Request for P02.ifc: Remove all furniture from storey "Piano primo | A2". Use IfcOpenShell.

First a look at what the model holds.

```python
import ifcopenshell
import ifcopenshell.util.element

model = ifcopenshell.open("P02.ifc")
print(model.schema)
storey = next(s for s in model.by_type("IfcBuildingStorey") if s.Name == "Piano primo | A2")
furniture = [e for e in ifcopenshell.util.element.get_decomposition(storey) if e.is_a("IfcFurnishingElement")]
seen = {}
for e in furniture:
    element_type = ifcopenshell.util.element.get_type(e)
    name = element_type.Name if element_type not in (None, e) else None
    seen[name] = seen.get(name, 0) + 1
for name, count in sorted(seen.items(), key=str):
    print(count, "x", name)
```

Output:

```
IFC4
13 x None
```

```python
import ifcopenshell
import ifcopenshell.api.root
import ifcopenshell.util.element

model = ifcopenshell.open("P02.ifc")

storey = next(s for s in model.by_type("IfcBuildingStorey") if s.Name == "Piano primo | A2")
furniture = [e for e in ifcopenshell.util.element.get_decomposition(storey) if e.is_a("IfcFurnishingElement")]

for e in furniture:
    ifcopenshell.api.root.remove_product(model, product=e)
print(len(furniture), "removed")

model.write("P02_edited.ifc")
```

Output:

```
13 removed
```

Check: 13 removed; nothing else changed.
